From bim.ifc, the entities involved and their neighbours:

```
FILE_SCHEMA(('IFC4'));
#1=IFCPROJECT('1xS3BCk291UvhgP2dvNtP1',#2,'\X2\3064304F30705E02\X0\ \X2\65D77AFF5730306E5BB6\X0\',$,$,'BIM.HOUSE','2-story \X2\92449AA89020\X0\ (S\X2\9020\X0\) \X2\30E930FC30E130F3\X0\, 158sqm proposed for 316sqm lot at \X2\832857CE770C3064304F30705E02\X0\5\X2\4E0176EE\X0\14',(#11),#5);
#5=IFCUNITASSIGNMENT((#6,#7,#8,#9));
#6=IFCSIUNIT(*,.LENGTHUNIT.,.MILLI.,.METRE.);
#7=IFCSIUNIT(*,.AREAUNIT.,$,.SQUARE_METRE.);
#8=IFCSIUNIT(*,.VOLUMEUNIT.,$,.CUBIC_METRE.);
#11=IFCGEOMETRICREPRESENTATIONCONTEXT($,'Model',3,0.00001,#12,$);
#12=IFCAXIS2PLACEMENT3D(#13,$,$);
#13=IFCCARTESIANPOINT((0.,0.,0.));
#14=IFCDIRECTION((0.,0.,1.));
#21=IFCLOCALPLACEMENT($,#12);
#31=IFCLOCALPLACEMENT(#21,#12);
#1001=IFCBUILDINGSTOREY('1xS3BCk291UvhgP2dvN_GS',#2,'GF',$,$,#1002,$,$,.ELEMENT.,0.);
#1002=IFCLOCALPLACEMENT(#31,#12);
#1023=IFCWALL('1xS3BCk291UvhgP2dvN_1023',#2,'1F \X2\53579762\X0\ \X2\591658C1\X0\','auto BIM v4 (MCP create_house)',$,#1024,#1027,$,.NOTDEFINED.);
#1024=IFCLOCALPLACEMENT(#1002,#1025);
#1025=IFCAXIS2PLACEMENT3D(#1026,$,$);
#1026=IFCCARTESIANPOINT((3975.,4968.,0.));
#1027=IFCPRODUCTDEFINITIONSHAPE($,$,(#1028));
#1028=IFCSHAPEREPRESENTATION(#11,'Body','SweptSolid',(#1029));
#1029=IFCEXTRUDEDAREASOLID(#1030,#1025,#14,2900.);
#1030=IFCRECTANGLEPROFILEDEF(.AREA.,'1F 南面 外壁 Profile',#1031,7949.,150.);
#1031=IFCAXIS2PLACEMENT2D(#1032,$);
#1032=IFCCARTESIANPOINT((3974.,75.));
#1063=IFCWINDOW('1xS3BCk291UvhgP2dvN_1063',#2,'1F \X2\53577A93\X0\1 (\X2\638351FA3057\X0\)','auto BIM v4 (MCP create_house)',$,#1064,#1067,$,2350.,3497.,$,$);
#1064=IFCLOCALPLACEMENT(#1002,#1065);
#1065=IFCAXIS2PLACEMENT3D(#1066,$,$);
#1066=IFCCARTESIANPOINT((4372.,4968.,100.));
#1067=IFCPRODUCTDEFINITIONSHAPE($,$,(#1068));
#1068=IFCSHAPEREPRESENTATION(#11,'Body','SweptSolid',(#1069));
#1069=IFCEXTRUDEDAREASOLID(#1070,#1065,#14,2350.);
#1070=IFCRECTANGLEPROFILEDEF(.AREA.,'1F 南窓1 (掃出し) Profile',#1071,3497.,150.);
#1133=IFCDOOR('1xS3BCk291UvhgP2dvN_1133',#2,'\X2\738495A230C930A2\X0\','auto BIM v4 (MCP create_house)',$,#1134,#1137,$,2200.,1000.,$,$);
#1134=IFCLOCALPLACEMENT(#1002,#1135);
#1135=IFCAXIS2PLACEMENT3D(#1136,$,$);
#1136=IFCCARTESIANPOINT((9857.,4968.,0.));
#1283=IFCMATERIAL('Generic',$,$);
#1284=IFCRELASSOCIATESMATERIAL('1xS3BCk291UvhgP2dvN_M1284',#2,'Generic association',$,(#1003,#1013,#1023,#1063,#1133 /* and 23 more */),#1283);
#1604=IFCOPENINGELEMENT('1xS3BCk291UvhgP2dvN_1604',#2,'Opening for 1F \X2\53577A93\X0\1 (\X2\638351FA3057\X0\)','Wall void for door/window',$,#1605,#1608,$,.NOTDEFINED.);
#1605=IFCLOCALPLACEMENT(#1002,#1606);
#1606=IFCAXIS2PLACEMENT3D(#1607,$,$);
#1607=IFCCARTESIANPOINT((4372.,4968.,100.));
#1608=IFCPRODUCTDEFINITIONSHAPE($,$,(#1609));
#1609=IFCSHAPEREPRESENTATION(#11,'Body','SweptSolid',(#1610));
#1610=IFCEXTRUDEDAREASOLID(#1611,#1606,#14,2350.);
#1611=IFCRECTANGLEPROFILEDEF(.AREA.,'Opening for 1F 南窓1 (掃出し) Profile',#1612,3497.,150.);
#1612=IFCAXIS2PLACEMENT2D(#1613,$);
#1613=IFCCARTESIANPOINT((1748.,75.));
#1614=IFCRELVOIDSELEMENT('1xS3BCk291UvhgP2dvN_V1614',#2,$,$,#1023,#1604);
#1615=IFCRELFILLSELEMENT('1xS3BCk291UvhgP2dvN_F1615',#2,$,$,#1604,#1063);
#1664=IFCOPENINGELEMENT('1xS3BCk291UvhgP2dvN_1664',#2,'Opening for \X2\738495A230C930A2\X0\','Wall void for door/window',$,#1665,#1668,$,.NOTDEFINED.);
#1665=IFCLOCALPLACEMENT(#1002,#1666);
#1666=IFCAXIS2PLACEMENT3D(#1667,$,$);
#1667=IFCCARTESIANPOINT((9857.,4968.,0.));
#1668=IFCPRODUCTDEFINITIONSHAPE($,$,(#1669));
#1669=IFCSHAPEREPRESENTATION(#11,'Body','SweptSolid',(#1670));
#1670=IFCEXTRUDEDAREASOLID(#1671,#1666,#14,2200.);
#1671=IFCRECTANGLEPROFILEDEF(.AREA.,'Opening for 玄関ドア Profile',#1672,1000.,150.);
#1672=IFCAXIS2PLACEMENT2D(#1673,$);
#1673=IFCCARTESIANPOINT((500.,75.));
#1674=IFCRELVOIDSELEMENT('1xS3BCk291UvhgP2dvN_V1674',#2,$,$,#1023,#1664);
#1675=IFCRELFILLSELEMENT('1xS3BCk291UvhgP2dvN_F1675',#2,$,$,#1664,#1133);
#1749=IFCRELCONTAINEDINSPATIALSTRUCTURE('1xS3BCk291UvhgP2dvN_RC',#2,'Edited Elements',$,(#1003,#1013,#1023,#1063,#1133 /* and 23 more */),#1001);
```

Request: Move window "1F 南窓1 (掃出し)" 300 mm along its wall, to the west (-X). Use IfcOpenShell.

```python
import ifcopenshell
import ifcopenshell.api.geometry
import ifcopenshell.util.placement
import ifcopenshell.util.unit

model = ifcopenshell.open("bim.ifc")
unit_scale = ifcopenshell.util.unit.calculate_unit_scale(model)

window = model.by_id(1063)
opening = window.FillsVoids[0].RelatingOpeningElement
wall = opening.VoidsElements[0].RelatingBuildingElement

wall_matrix = ifcopenshell.util.placement.get_local_placement(wall.ObjectPlacement)
shift = wall_matrix[:3, 0] * -0.3 / unit_scale
before = ifcopenshell.util.placement.get_local_placement(window.ObjectPlacement)[:3, 3].copy()

# The window is not placed relative to its opening, so move both.
for product in (opening, window):
    matrix = ifcopenshell.util.placement.get_local_placement(product.ObjectPlacement)
    matrix[:3, 3] += shift
    ifcopenshell.api.geometry.edit_object_placement(model, product=product, matrix=matrix, is_si=False)

after = ifcopenshell.util.placement.get_local_placement(window.ObjectPlacement)[:3, 3]
print("window moved by", (after - before).round(3) + 0.0)

model.write("bim_rev.ifc")
```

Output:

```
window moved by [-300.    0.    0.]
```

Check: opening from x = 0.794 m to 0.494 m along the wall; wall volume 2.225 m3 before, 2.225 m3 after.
